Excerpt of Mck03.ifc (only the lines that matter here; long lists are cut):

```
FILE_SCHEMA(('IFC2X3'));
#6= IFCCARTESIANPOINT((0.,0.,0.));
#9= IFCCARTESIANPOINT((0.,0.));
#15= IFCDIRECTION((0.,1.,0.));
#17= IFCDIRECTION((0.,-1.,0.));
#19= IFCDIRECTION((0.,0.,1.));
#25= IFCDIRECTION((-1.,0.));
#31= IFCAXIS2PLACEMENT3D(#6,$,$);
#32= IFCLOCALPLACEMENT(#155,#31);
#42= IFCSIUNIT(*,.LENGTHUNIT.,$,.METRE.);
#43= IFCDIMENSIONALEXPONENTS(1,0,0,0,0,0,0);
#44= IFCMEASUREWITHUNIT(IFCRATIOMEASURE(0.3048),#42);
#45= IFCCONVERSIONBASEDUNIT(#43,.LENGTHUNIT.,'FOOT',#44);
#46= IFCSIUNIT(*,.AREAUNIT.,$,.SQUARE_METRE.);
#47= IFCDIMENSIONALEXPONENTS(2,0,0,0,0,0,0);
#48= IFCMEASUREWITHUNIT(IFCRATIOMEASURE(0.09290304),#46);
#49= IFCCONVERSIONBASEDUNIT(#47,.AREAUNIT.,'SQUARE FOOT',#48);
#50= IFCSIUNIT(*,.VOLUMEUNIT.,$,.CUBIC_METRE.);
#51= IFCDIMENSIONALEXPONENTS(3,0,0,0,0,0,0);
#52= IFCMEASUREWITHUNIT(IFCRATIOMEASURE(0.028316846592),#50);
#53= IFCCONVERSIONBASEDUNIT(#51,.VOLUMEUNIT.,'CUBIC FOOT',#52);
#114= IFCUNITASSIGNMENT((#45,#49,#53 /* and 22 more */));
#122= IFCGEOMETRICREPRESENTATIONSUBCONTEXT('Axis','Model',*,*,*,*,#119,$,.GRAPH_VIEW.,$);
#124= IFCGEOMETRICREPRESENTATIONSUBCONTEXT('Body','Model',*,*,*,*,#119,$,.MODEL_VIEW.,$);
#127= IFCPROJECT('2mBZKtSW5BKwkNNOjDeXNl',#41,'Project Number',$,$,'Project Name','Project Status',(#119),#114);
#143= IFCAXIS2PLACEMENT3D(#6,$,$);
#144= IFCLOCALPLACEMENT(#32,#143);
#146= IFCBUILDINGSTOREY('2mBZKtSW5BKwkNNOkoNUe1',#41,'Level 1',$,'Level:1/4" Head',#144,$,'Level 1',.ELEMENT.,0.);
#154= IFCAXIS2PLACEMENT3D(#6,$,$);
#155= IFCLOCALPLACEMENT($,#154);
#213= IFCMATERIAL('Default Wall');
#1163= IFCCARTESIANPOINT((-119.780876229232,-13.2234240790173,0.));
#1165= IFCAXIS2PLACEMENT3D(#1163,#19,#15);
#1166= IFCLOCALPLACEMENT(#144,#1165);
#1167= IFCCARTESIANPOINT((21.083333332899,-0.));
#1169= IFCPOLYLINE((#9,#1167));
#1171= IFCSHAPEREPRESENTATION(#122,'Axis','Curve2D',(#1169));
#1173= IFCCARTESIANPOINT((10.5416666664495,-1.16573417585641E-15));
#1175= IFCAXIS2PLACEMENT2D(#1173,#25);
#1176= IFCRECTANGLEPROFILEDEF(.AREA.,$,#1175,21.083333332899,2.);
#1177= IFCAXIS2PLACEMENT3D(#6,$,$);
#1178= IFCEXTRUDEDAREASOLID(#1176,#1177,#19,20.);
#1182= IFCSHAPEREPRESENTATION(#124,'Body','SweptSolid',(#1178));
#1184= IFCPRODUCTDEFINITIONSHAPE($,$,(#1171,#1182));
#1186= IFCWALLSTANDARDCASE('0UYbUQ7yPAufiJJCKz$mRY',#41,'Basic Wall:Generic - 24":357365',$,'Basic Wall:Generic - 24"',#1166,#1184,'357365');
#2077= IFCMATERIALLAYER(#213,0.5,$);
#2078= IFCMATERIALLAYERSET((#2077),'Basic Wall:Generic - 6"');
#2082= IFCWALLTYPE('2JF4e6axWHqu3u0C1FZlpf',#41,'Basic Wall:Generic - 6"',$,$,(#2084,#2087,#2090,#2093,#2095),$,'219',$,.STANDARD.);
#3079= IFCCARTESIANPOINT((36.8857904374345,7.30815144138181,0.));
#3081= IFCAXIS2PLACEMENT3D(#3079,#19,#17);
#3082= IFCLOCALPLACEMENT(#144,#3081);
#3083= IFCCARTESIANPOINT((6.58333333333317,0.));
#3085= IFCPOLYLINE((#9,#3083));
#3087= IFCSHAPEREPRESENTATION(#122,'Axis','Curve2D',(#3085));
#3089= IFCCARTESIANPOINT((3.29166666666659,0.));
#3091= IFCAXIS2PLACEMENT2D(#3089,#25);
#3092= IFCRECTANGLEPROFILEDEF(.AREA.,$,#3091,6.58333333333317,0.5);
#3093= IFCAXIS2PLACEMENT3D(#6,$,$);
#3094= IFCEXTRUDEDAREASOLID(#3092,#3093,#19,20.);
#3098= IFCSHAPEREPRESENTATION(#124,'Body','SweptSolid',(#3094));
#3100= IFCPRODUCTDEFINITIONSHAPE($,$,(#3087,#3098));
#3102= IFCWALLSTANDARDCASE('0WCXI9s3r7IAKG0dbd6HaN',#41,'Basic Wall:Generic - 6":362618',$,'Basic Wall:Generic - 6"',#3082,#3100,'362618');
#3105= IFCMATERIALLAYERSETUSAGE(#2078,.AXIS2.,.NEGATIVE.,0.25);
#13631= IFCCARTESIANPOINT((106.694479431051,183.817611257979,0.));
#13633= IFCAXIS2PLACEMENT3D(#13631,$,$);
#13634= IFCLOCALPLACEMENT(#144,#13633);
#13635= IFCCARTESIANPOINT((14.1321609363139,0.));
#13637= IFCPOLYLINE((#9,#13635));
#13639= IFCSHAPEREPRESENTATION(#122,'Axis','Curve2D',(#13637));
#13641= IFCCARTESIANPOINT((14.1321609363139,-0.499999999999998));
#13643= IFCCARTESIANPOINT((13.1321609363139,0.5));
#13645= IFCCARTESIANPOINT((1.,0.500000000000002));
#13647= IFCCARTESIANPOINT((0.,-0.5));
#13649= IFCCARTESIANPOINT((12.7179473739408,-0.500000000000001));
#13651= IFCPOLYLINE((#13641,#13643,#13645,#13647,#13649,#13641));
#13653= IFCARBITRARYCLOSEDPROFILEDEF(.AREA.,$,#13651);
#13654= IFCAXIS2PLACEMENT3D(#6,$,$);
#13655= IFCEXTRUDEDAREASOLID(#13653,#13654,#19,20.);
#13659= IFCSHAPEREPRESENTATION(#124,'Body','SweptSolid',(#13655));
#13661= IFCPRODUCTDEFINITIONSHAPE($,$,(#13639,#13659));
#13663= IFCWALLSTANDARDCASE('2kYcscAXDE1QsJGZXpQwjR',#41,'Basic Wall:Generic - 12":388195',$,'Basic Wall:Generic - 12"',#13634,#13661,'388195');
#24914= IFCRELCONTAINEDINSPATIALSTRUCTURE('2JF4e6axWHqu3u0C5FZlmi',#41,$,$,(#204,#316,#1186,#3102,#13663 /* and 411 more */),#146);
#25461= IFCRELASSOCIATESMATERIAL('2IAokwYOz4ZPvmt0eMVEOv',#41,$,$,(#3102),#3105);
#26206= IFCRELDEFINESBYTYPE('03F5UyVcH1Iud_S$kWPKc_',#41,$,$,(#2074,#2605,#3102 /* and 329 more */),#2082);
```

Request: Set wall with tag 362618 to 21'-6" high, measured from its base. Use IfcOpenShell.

```python
import ifcopenshell
import ifcopenshell.geom
import ifcopenshell.util.representation
import ifcopenshell.util.shape
import ifcopenshell.util.unit

model = ifcopenshell.open("Mck03.ifc")
unit_scale = ifcopenshell.util.unit.calculate_unit_scale(model)
settings = ifcopenshell.geom.settings()


def volume(element):
    """Net volume in cubic metres, openings subtracted."""
    shape = ifcopenshell.geom.create_shape(settings, element)
    return ifcopenshell.util.shape.get_volume(shape.geometry)


wall = model.by_guid("0WCXI9s3r7IAKG0dbd6HaN")
before = volume(wall)

body = ifcopenshell.util.representation.get_representation(wall, "Model", "Body")
solid = body.Items[0]
old_height = solid.Depth
solid.Depth = 258 * 0.0254 / unit_scale
after = volume(wall)

print(f"height {old_height:g} -> {solid.Depth:g}, volume {before:.3f} -> {after:.3f} m3")

model.write("Mck03-out.ifc")
```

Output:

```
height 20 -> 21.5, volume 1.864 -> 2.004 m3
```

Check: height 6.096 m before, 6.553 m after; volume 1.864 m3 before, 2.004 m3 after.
